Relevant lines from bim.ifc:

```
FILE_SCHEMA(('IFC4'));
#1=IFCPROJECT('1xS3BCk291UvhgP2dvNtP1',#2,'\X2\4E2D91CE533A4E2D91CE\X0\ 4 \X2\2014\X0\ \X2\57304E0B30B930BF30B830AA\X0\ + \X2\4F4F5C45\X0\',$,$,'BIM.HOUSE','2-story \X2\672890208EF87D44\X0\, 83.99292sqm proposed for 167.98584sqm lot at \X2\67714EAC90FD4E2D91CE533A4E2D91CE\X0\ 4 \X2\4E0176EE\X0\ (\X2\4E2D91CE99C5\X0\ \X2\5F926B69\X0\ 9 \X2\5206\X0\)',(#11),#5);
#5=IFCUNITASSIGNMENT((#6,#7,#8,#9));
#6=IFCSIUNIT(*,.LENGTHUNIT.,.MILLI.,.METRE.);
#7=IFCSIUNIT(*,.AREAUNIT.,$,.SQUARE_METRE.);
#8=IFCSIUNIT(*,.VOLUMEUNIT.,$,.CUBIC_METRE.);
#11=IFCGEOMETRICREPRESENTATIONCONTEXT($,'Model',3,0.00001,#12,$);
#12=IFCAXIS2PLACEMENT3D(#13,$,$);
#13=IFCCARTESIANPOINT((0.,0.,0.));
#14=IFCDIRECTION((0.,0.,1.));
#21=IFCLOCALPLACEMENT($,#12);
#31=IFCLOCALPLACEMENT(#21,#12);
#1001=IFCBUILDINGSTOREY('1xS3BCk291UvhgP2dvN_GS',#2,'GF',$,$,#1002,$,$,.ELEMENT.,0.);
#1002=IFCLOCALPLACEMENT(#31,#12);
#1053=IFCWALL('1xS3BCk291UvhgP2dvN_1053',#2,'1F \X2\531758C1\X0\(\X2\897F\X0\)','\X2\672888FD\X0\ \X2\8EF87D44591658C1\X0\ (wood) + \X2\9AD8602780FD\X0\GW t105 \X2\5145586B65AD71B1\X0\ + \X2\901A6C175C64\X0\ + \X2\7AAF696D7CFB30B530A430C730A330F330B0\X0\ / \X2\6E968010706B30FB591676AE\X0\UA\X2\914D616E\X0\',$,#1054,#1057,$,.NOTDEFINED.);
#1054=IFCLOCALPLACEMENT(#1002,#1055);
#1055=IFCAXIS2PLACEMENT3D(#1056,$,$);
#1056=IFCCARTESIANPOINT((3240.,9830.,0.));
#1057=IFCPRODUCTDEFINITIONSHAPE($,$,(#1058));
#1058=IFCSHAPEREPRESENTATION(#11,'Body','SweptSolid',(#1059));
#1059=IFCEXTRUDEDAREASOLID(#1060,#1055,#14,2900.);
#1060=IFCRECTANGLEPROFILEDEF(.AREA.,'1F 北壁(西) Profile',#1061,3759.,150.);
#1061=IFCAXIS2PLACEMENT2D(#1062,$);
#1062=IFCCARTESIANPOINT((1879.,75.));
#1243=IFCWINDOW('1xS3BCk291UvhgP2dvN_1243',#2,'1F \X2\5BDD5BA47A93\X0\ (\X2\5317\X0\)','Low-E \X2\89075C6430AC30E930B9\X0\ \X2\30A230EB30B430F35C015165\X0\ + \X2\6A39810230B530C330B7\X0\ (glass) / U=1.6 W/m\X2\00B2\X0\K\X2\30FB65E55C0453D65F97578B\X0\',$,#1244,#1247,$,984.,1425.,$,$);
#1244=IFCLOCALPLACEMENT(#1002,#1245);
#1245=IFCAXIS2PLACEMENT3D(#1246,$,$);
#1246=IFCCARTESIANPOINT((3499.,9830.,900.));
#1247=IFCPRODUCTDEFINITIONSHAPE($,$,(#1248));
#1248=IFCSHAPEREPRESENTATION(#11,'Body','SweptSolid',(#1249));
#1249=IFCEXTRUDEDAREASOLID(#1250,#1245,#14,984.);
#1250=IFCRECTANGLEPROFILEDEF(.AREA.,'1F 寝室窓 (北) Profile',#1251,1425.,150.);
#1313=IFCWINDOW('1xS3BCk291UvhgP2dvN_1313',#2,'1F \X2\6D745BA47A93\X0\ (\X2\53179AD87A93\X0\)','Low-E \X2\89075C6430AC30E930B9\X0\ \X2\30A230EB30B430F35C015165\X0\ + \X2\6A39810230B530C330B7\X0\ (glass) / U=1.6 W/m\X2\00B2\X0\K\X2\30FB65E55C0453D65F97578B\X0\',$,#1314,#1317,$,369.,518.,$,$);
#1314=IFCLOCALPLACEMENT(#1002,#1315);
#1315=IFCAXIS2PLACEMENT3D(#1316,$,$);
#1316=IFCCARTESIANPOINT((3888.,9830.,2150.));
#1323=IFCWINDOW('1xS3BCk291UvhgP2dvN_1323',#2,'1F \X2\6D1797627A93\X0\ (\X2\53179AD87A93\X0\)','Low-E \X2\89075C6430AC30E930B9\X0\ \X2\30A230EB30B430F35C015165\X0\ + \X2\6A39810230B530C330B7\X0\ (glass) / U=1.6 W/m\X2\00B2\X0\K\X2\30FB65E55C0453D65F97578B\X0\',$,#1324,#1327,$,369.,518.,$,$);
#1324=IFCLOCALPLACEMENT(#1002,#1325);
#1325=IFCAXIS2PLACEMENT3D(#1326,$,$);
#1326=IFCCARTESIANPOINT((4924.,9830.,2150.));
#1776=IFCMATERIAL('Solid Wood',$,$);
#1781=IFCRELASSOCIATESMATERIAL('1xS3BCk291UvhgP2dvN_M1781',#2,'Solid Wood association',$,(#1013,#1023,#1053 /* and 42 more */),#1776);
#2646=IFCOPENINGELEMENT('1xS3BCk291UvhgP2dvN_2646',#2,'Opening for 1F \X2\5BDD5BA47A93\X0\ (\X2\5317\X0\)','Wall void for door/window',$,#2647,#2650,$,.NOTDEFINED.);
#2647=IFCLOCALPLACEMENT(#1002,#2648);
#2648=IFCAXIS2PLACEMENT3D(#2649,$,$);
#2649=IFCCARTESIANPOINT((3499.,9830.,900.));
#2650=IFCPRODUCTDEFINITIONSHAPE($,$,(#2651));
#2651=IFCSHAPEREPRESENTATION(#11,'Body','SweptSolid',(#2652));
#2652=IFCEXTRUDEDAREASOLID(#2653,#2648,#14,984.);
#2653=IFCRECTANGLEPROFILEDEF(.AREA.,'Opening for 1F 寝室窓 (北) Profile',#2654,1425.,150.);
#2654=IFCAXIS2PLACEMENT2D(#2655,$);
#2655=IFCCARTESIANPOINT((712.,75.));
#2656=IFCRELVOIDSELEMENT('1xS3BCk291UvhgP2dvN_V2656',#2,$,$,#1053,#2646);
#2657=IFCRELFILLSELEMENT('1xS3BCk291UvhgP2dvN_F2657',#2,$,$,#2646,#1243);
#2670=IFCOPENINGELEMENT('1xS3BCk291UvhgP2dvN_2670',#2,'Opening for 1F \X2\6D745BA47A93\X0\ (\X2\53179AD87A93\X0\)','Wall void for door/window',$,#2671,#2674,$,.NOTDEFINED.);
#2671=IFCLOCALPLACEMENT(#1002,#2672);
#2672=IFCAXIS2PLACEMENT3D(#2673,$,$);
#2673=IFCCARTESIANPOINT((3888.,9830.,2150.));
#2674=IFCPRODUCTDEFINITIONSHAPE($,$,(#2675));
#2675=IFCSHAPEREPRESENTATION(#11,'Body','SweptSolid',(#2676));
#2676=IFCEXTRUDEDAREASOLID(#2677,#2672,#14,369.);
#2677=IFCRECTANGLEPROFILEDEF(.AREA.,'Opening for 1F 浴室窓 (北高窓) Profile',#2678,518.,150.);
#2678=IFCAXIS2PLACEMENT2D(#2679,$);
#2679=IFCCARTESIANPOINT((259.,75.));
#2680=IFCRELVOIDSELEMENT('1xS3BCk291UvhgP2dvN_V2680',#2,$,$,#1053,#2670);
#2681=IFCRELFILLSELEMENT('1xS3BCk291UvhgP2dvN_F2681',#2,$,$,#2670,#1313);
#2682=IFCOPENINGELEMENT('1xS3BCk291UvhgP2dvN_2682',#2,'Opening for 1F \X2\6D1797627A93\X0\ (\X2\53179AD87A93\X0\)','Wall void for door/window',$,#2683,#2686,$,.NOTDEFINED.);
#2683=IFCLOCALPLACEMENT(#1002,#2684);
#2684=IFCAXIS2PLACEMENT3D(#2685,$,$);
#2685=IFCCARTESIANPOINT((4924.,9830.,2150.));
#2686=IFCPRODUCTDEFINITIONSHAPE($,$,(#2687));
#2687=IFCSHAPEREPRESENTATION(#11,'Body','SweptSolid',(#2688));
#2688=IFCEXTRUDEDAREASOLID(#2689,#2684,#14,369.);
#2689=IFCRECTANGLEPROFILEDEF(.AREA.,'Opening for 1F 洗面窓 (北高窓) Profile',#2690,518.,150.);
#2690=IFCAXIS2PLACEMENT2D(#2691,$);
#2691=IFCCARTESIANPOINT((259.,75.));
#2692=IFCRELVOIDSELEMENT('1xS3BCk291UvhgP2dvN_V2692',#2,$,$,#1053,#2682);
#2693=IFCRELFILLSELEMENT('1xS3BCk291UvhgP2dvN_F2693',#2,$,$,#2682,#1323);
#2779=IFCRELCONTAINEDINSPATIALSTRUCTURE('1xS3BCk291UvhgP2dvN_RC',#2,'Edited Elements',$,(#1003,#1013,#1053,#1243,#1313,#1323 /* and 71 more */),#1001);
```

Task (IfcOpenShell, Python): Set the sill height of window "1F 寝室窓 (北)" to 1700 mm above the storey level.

```python
import numpy as np
import ifcopenshell
import ifcopenshell.api.geometry
import ifcopenshell.geom
import ifcopenshell.util.element
import ifcopenshell.util.placement
import ifcopenshell.util.shape
import ifcopenshell.util.unit

model = ifcopenshell.open("bim.ifc")
unit_scale = ifcopenshell.util.unit.calculate_unit_scale(model)

window = model.by_guid("1xS3BCk291UvhgP2dvN_1243")
opening = window.FillsVoids[0].RelatingOpeningElement
storey = ifcopenshell.util.element.get_container(window, ifc_class="IfcBuildingStorey")
level = ifcopenshell.util.placement.get_local_placement(storey.ObjectPlacement)[2, 3]

# The opening's origin need not be at the sill, so measure its lowest point.
shape = ifcopenshell.geom.create_shape(ifcopenshell.geom.settings(), opening)
bottom = ifcopenshell.util.shape.get_shape_bottom_elevation(shape, shape.geometry) / unit_scale
dz = level + 1700.0 - bottom

shift = np.array([0.0, 0.0, dz])
# The window is not placed relative to its opening, so move both.
for product in (opening, window):
    matrix = ifcopenshell.util.placement.get_local_placement(product.ObjectPlacement)
    matrix[:3, 3] += shift
    ifcopenshell.api.geometry.edit_object_placement(model, product=product, matrix=matrix, is_si=False)

print(f"moved by {dz * unit_scale:+.3f} m")

model.write("bim_edited.ifc")
```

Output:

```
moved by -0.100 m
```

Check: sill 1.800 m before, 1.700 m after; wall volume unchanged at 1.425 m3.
